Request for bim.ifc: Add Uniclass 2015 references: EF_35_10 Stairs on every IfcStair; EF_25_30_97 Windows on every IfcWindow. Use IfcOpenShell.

First a look at what the model holds.

```python
import ifcopenshell

model = ifcopenshell.open("bim.ifc")
print(model.schema)
print("classifications:", [c.Name for c in model.by_type("IfcClassification")])
for ifc_class in ("IfcDoor", "IfcRoof", "IfcStair", "IfcWall", "IfcWindow"):
    print(ifc_class, len(model.by_type(ifc_class)))
```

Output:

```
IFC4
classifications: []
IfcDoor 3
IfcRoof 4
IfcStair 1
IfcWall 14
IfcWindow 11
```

```python
import ifcopenshell
import ifcopenshell.api.classification

model = ifcopenshell.open("bim.ifc")

system = ifcopenshell.api.classification.add_classification(model, classification="Uniclass 2015")

codes = {
    "IfcStair": ("EF_35_10", "Stairs"),
    "IfcWindow": ("EF_25_30_97", "Windows"),
}
for ifc_class, (code, name) in codes.items():
    products = model.by_type(ifc_class)
    ifcopenshell.api.classification.add_reference(
        model, products=products, classification=system, identification=code, name=name
    )
    print(code, len(products))

model.write("bim-out.ifc")
```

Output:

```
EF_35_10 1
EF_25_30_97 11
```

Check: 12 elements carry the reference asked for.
